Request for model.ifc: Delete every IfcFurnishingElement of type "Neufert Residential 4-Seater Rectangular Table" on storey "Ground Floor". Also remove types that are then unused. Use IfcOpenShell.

First a look at what the model holds.

```python
import ifcopenshell
import ifcopenshell.util.element

model = ifcopenshell.open("model.ifc")
print(model.schema)
storey = next(s for s in model.by_type("IfcBuildingStorey") if s.Name == "Ground Floor")
furniture = [e for e in ifcopenshell.util.element.get_decomposition(storey) if e.is_a("IfcFurnishingElement")]
seen = {}
for e in furniture:
    element_type = ifcopenshell.util.element.get_type(e)
    name = element_type.Name if element_type not in (None, e) else None
    seen[name] = seen.get(name, 0) + 1
for name, count in sorted(seen.items(), key=str):
    print(count, "x", name)
```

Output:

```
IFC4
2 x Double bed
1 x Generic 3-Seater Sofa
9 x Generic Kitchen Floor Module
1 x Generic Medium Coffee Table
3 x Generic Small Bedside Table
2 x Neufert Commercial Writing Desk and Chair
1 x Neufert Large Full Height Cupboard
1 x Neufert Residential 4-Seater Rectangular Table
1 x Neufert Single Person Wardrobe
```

```python
import ifcopenshell
import ifcopenshell.api.root
import ifcopenshell.util.element

model = ifcopenshell.open("model.ifc")

storey = next(s for s in model.by_type("IfcBuildingStorey") if s.Name == "Ground Floor")
furniture = [e for e in ifcopenshell.util.element.get_decomposition(storey) if e.is_a("IfcFurnishingElement")]
targets = [e for e in furniture if (t := ifcopenshell.util.element.get_type(e)) not in (None, e) and t.Name == "Neufert Residential 4-Seater Rectangular Table"]
types = {ifcopenshell.util.element.get_type(e) for e in targets} - {None, *targets}

for e in targets:
    ifcopenshell.api.root.remove_product(model, product=e)
print(len(targets), "removed")

unused = [t for t in types if not ifcopenshell.util.element.get_types(t)]
for t in unused:
    ifcopenshell.api.root.remove_product(model, product=t)
print(len(unused), "unused types removed")

model.write("model_rev.ifc")
```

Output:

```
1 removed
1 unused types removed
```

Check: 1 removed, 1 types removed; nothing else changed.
